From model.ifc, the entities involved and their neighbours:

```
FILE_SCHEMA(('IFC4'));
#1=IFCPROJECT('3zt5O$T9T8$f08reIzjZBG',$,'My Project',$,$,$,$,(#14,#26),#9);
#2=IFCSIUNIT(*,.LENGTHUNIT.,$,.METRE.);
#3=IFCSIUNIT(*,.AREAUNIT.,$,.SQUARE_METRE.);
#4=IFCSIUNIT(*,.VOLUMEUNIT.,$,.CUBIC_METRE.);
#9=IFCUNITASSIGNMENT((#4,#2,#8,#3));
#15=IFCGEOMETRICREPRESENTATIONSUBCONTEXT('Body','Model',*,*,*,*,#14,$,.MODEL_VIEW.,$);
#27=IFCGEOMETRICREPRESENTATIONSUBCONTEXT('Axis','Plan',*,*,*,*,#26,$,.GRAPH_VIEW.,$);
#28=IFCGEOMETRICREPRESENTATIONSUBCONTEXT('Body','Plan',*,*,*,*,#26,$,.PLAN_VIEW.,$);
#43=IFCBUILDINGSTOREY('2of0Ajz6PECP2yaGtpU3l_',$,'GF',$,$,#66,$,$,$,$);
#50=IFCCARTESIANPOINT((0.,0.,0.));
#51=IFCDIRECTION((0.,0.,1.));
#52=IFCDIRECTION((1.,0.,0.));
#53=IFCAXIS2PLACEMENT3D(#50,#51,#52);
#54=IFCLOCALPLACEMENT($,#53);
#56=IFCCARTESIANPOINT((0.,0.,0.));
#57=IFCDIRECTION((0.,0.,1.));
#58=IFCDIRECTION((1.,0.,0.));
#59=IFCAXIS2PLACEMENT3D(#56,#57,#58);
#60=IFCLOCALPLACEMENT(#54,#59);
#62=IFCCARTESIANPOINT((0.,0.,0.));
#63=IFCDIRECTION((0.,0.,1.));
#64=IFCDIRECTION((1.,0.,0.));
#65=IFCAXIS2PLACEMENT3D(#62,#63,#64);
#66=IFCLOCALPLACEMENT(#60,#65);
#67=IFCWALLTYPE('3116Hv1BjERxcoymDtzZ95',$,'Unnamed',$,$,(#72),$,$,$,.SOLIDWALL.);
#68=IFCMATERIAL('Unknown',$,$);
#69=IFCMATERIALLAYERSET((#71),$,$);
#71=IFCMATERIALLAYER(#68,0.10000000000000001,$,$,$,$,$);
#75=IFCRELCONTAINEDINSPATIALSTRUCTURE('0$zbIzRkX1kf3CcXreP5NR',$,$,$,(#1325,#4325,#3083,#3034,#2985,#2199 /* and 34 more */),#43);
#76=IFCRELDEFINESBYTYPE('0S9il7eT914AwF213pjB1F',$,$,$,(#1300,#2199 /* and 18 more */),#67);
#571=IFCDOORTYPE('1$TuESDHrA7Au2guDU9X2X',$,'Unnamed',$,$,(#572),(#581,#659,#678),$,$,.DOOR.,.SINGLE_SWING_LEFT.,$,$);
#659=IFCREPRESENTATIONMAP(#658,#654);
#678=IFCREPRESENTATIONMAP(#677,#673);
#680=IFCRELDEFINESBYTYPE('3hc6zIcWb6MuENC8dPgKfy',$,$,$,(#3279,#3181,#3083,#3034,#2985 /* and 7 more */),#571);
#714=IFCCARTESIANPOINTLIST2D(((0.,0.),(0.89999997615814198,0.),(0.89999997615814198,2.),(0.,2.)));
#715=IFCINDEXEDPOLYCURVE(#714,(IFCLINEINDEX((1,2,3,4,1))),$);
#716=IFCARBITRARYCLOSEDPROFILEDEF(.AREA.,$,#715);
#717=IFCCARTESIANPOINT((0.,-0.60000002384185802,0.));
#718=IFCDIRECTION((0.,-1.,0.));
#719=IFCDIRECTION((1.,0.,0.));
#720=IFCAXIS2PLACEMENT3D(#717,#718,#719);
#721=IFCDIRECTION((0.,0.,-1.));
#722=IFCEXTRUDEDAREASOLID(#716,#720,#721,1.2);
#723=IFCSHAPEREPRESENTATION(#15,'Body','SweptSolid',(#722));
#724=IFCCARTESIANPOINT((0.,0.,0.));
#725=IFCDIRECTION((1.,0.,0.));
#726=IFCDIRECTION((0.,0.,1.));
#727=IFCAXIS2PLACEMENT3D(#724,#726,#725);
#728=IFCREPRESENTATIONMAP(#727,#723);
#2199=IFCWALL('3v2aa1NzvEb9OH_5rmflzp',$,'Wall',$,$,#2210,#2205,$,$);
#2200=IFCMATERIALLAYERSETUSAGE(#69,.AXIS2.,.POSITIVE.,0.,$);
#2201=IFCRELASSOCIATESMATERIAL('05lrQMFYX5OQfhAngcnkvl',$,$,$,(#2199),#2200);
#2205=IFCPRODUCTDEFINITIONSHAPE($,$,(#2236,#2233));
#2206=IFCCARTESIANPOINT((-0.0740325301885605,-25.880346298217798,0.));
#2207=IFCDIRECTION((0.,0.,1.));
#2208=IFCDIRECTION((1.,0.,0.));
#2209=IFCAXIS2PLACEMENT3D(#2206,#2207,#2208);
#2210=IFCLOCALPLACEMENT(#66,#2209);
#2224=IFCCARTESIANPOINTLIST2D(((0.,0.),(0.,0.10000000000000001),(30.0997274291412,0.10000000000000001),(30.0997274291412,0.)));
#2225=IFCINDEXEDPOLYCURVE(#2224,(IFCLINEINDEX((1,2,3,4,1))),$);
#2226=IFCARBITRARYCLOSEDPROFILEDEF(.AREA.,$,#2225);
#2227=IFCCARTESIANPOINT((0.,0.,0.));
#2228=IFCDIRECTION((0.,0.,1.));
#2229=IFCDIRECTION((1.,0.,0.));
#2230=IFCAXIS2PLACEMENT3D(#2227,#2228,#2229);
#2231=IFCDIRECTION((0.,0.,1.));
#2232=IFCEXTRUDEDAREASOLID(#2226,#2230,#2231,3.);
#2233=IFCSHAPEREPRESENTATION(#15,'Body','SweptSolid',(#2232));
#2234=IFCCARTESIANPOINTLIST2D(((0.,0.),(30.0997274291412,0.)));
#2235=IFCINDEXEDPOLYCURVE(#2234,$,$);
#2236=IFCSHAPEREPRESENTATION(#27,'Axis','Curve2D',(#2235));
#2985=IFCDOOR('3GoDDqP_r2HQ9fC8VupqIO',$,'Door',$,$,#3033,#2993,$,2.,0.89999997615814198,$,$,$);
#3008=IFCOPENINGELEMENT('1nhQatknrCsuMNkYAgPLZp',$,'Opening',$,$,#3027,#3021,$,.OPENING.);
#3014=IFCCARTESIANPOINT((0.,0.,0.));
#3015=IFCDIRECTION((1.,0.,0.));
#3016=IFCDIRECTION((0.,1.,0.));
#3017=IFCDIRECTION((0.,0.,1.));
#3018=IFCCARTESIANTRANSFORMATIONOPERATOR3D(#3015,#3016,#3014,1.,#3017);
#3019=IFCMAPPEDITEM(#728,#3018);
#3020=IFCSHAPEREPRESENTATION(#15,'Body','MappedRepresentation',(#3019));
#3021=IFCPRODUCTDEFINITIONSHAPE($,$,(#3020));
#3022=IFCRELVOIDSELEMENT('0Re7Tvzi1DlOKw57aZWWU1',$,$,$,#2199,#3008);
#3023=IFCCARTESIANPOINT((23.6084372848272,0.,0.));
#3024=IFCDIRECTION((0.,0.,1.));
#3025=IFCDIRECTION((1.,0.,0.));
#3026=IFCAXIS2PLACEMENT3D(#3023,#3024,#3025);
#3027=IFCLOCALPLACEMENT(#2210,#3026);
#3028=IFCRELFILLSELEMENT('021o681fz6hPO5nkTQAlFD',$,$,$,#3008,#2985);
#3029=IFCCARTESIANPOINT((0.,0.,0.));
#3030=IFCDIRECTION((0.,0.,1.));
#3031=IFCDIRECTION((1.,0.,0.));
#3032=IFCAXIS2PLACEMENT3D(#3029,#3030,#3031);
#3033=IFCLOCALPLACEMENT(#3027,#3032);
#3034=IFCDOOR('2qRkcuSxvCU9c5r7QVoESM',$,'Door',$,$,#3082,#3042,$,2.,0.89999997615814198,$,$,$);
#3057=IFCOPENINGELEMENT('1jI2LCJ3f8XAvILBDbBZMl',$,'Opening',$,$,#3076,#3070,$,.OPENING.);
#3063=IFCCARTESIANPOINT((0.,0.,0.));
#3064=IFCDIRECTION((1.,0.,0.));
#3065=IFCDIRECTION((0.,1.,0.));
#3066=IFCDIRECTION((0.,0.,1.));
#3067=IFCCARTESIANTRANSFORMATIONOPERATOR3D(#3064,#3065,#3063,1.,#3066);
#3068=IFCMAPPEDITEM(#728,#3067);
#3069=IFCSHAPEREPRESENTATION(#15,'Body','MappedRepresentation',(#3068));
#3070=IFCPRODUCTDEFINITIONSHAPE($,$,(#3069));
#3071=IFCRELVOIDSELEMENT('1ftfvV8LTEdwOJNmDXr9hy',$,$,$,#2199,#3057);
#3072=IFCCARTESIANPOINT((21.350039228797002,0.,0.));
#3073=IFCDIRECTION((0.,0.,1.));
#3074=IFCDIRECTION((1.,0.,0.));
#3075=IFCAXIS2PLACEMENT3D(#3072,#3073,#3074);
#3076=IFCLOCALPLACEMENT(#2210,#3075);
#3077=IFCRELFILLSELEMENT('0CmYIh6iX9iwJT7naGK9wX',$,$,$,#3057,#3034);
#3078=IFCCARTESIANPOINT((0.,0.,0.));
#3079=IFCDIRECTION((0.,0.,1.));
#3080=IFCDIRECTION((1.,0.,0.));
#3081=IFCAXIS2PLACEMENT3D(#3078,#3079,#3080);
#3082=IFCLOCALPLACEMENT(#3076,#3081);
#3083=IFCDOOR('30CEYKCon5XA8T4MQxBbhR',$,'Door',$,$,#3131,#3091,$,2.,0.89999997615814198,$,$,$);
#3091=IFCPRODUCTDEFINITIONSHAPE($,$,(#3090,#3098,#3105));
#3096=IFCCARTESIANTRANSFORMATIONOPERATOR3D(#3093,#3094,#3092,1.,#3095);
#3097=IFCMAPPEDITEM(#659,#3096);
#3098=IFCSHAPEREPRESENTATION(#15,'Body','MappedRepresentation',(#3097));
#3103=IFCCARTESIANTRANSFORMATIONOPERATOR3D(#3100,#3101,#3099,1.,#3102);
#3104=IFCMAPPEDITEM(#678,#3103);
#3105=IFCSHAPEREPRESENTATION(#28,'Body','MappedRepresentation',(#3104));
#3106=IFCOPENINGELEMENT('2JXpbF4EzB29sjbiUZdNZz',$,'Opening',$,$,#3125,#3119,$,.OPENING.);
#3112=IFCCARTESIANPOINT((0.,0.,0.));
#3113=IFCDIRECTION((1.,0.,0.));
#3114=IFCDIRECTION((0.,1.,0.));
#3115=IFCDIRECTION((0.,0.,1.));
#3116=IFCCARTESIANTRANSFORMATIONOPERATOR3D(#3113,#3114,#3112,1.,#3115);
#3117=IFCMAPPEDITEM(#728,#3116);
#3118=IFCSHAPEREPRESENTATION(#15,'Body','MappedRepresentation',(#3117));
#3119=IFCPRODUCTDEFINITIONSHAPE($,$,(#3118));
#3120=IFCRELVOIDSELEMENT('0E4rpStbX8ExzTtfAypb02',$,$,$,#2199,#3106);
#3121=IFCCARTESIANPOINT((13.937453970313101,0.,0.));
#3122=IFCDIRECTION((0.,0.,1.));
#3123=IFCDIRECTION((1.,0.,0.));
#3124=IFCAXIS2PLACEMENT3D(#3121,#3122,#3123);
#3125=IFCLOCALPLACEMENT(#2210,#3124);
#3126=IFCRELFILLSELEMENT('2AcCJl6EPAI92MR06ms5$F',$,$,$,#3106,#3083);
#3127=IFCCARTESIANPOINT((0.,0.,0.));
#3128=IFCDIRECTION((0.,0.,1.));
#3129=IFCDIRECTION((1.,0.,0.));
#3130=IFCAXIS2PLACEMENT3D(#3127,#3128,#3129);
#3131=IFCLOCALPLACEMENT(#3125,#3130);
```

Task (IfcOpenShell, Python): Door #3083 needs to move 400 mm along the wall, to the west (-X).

```python
import ifcopenshell
import ifcopenshell.api.geometry
import ifcopenshell.util.placement
import ifcopenshell.util.unit

model = ifcopenshell.open("model.ifc")
unit_scale = ifcopenshell.util.unit.calculate_unit_scale(model)

door = model.by_guid("30CEYKCon5XA8T4MQxBbhR")
opening = door.FillsVoids[0].RelatingOpeningElement
wall = opening.VoidsElements[0].RelatingBuildingElement

wall_matrix = ifcopenshell.util.placement.get_local_placement(wall.ObjectPlacement)
shift = wall_matrix[:3, 0] * -0.4 / unit_scale
before = ifcopenshell.util.placement.get_local_placement(door.ObjectPlacement)[:3, 3].copy()

# The door is placed relative to its opening, so it follows when the opening moves.
matrix = ifcopenshell.util.placement.get_local_placement(opening.ObjectPlacement)
matrix[:3, 3] += shift
ifcopenshell.api.geometry.edit_object_placement(
    model, product=opening, matrix=matrix, is_si=False, should_transform_children=True
)

after = ifcopenshell.util.placement.get_local_placement(door.ObjectPlacement)[:3, 3]
print("door moved by", (after - before).round(3) + 0.0)

model.write("model_updated.ifc")
```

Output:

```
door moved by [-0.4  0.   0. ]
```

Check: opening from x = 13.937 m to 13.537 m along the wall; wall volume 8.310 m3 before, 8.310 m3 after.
